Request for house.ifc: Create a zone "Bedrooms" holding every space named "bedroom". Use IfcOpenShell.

First a look at what the model holds.

```python
import ifcopenshell

model = ifcopenshell.open("house.ifc")
print(model.schema)
seen = {}
for space in model.by_type("IfcSpace"):
    seen[space.LongName] = seen.get(space.LongName, 0) + 1
for name, count in sorted(seen.items(), key=str):
    print(count, "x", name)
print("zones:", [z.Name for z in model.by_type("IfcZone")][:20])
```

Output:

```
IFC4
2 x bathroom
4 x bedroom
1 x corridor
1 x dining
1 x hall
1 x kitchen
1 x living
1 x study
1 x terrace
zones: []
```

```python
import ifcopenshell
import ifcopenshell.api.group
import ifcopenshell.api.root

model = ifcopenshell.open("house.ifc")

names = {"bedroom"}
spaces = [s for s in model.by_type("IfcSpace") if s.LongName in names]

zone = ifcopenshell.api.root.create_entity(model, ifc_class="IfcZone", name="Bedrooms")
ifcopenshell.api.group.assign_group(model, products=spaces, group=zone)
print(len(spaces), "spaces in", zone.Name)

model.write("house_updated.ifc")
```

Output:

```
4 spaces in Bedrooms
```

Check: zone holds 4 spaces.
